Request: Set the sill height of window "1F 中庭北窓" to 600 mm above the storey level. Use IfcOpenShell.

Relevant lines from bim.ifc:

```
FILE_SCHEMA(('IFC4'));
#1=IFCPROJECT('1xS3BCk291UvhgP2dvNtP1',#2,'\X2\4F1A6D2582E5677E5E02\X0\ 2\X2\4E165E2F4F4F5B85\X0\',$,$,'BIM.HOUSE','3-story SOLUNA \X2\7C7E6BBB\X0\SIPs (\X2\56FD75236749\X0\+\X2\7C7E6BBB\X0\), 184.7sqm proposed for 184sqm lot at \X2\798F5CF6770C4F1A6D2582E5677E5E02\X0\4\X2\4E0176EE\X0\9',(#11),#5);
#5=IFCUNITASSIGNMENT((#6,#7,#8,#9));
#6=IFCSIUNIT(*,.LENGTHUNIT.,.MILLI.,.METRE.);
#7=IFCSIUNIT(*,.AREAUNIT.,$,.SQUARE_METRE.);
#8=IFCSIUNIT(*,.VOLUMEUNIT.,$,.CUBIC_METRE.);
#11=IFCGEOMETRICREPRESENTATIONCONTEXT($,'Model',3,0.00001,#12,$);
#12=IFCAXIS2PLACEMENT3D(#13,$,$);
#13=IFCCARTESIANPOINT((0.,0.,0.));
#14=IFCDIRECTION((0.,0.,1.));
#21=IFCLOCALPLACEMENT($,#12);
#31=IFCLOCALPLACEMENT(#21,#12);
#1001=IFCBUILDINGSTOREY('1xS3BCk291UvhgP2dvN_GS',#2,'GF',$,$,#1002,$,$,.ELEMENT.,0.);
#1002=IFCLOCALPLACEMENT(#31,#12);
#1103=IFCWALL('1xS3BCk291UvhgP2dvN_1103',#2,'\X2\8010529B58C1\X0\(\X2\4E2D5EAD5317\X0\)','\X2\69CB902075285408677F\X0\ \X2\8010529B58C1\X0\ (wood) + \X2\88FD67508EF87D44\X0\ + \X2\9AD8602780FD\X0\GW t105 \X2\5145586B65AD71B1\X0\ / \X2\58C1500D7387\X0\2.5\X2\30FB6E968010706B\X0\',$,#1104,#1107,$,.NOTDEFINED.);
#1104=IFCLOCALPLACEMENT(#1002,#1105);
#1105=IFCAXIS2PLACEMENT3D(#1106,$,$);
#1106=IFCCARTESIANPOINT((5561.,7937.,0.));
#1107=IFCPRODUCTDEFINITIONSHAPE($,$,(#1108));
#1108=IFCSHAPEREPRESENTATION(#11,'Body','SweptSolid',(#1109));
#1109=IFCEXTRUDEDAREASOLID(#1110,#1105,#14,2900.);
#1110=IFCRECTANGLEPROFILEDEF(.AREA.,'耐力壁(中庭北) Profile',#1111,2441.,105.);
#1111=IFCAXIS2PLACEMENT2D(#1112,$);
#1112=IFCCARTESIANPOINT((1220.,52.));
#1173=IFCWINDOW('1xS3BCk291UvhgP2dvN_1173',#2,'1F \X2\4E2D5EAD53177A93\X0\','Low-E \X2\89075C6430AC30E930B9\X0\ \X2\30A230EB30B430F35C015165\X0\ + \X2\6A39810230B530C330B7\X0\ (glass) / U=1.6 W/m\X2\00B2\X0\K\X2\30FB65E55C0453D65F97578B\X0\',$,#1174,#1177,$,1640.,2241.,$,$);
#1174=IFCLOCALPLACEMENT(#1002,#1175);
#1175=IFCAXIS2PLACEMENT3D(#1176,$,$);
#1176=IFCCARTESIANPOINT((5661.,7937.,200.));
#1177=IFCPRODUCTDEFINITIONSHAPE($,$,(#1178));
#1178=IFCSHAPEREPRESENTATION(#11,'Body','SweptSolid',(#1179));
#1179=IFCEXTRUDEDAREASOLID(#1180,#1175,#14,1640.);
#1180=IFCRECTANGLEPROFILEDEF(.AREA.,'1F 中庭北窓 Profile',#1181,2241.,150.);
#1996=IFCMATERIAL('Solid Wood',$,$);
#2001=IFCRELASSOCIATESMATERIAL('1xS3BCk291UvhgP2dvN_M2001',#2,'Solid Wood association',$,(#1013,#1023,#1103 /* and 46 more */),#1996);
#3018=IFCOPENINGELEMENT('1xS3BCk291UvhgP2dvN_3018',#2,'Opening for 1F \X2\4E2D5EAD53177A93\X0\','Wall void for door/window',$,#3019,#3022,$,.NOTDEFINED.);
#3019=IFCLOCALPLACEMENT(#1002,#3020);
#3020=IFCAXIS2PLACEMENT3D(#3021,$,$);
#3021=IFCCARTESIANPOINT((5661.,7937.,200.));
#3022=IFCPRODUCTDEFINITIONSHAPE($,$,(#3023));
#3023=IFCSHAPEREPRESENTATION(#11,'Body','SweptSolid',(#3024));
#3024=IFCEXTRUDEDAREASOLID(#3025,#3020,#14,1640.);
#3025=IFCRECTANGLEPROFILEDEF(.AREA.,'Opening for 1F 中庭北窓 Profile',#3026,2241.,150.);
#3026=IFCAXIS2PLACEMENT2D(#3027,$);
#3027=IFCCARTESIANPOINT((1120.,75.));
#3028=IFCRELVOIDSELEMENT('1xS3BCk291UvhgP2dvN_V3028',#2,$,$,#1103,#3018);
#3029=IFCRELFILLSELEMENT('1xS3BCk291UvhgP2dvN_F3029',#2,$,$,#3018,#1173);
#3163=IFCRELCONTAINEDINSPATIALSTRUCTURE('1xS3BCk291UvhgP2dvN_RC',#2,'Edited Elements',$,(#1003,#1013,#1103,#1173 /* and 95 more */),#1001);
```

```python
import numpy as np
import ifcopenshell
import ifcopenshell.api.geometry
import ifcopenshell.geom
import ifcopenshell.util.element
import ifcopenshell.util.placement
import ifcopenshell.util.shape
import ifcopenshell.util.unit

model = ifcopenshell.open("bim.ifc")
unit_scale = ifcopenshell.util.unit.calculate_unit_scale(model)

window = model.by_guid("1xS3BCk291UvhgP2dvN_1173")
opening = window.FillsVoids[0].RelatingOpeningElement
storey = ifcopenshell.util.element.get_container(window, ifc_class="IfcBuildingStorey")
level = ifcopenshell.util.placement.get_local_placement(storey.ObjectPlacement)[2, 3]

# The opening's origin need not be at the sill, so measure its lowest point.
shape = ifcopenshell.geom.create_shape(ifcopenshell.geom.settings(), opening)
bottom = ifcopenshell.util.shape.get_shape_bottom_elevation(shape, shape.geometry) / unit_scale
dz = level + 600.0 - bottom

shift = np.array([0.0, 0.0, dz])
# The window is not placed relative to its opening, so move both.
for product in (opening, window):
    matrix = ifcopenshell.util.placement.get_local_placement(product.ObjectPlacement)
    matrix[:3, 3] += shift
    ifcopenshell.api.geometry.edit_object_placement(model, product=product, matrix=matrix, is_si=False)

print(f"moved by {dz * unit_scale:+.3f} m")

model.write("bim_rev.ifc")
```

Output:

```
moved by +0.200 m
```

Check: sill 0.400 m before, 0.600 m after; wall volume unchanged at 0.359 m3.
